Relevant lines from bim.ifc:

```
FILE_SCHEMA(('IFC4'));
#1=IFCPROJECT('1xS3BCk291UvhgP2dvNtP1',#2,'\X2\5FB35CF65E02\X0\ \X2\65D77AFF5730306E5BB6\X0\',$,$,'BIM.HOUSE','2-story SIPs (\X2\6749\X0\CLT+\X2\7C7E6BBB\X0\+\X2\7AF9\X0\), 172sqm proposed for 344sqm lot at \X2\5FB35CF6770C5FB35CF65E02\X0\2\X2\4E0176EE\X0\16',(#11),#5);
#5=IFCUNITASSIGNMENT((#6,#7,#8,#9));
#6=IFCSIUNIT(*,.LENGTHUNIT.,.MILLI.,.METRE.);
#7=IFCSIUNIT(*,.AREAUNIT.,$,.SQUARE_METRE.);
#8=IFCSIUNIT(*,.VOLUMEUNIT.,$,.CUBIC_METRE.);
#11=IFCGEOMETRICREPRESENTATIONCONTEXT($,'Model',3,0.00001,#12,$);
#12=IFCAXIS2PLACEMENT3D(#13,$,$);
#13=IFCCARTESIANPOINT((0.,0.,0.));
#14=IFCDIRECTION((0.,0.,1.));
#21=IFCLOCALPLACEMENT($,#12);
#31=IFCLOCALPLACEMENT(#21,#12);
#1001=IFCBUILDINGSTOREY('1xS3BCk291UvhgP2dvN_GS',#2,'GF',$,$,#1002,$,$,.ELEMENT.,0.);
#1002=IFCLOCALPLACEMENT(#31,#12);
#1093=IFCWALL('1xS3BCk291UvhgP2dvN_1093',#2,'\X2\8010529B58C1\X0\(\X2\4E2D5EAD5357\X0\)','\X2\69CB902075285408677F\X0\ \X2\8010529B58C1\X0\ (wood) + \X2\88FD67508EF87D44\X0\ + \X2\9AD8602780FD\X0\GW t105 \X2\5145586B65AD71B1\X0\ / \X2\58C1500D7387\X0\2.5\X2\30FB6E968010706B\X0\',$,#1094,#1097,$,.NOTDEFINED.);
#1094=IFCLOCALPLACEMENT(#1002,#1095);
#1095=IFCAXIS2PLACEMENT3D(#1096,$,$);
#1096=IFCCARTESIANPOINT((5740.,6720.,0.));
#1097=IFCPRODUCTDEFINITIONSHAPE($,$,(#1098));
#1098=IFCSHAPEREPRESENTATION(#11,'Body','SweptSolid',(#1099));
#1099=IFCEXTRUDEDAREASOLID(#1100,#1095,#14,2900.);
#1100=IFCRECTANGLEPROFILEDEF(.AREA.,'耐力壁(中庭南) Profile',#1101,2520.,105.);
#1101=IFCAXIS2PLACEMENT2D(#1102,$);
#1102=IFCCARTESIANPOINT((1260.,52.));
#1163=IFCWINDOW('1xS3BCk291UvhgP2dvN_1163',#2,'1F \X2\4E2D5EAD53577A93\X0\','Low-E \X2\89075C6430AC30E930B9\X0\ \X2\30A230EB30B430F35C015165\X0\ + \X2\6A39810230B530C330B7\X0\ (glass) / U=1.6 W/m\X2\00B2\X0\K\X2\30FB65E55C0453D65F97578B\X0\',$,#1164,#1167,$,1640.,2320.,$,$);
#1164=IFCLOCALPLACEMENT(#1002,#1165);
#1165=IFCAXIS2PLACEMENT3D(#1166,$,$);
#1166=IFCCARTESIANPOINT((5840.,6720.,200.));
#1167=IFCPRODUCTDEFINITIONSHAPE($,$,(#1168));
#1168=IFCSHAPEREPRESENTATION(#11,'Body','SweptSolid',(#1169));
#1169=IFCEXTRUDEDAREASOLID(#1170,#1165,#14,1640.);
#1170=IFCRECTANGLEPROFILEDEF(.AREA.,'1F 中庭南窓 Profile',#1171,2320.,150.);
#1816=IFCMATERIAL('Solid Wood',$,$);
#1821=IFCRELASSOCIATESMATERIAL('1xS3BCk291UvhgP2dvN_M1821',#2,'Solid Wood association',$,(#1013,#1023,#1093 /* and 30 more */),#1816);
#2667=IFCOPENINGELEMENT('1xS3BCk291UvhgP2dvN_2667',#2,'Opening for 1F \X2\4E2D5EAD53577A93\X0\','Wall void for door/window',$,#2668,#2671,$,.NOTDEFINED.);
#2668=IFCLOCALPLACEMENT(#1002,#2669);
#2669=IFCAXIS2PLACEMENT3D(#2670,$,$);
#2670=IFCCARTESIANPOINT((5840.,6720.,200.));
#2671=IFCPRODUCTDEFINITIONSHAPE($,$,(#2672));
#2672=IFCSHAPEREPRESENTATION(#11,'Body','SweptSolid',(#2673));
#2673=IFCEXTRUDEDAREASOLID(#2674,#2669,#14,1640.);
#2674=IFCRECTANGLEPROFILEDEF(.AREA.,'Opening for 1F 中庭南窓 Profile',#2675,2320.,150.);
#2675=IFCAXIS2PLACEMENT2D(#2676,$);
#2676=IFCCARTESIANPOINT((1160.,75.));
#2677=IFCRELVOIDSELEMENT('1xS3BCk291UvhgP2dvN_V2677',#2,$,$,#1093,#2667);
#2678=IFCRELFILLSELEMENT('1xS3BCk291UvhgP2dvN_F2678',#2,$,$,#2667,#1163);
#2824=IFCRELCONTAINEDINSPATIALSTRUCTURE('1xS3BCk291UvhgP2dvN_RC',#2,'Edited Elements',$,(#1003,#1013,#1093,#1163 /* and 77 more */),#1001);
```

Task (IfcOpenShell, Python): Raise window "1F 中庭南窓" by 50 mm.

```python
import numpy as np
import ifcopenshell
import ifcopenshell.api.geometry
import ifcopenshell.util.placement
import ifcopenshell.util.unit

model = ifcopenshell.open("bim.ifc")
unit_scale = ifcopenshell.util.unit.calculate_unit_scale(model)

window = model.by_guid("1xS3BCk291UvhgP2dvN_1163")
opening = window.FillsVoids[0].RelatingOpeningElement
dz = 0.05 / unit_scale

shift = np.array([0.0, 0.0, dz])
# The window is not placed relative to its opening, so move both.
for product in (opening, window):
    matrix = ifcopenshell.util.placement.get_local_placement(product.ObjectPlacement)
    matrix[:3, 3] += shift
    ifcopenshell.api.geometry.edit_object_placement(model, product=product, matrix=matrix, is_si=False)

print(f"moved by {dz * unit_scale:+.3f} m")

model.write("bim_updated.ifc")
```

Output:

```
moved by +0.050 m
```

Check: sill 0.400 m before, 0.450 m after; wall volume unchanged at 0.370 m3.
